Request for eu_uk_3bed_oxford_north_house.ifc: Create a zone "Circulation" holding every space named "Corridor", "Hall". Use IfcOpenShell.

First a look at what the model holds.

```python
import ifcopenshell

model = ifcopenshell.open("eu_uk_3bed_oxford_north_house.ifc")
print(model.schema)
seen = {}
for space in model.by_type("IfcSpace"):
    seen[space.LongName] = seen.get(space.LongName, 0) + 1
for name, count in sorted(seen.items(), key=str):
    print(count, "x", name)
print("zones:", [z.Name for z in model.by_type("IfcZone")][:20])
```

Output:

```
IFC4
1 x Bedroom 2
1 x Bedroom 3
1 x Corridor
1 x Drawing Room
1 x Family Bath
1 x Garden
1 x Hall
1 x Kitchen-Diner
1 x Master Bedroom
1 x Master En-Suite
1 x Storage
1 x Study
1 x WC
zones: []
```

```python
import ifcopenshell
import ifcopenshell.api.group
import ifcopenshell.api.root

model = ifcopenshell.open("eu_uk_3bed_oxford_north_house.ifc")

names = {"Corridor", "Hall"}
spaces = [s for s in model.by_type("IfcSpace") if s.LongName in names]

zone = ifcopenshell.api.root.create_entity(model, ifc_class="IfcZone", name="Circulation")
ifcopenshell.api.group.assign_group(model, products=spaces, group=zone)
print(len(spaces), "spaces in", zone.Name)

model.write("eu_uk_3bed_oxford_north_house-out.ifc")
```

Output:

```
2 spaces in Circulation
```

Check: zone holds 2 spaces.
